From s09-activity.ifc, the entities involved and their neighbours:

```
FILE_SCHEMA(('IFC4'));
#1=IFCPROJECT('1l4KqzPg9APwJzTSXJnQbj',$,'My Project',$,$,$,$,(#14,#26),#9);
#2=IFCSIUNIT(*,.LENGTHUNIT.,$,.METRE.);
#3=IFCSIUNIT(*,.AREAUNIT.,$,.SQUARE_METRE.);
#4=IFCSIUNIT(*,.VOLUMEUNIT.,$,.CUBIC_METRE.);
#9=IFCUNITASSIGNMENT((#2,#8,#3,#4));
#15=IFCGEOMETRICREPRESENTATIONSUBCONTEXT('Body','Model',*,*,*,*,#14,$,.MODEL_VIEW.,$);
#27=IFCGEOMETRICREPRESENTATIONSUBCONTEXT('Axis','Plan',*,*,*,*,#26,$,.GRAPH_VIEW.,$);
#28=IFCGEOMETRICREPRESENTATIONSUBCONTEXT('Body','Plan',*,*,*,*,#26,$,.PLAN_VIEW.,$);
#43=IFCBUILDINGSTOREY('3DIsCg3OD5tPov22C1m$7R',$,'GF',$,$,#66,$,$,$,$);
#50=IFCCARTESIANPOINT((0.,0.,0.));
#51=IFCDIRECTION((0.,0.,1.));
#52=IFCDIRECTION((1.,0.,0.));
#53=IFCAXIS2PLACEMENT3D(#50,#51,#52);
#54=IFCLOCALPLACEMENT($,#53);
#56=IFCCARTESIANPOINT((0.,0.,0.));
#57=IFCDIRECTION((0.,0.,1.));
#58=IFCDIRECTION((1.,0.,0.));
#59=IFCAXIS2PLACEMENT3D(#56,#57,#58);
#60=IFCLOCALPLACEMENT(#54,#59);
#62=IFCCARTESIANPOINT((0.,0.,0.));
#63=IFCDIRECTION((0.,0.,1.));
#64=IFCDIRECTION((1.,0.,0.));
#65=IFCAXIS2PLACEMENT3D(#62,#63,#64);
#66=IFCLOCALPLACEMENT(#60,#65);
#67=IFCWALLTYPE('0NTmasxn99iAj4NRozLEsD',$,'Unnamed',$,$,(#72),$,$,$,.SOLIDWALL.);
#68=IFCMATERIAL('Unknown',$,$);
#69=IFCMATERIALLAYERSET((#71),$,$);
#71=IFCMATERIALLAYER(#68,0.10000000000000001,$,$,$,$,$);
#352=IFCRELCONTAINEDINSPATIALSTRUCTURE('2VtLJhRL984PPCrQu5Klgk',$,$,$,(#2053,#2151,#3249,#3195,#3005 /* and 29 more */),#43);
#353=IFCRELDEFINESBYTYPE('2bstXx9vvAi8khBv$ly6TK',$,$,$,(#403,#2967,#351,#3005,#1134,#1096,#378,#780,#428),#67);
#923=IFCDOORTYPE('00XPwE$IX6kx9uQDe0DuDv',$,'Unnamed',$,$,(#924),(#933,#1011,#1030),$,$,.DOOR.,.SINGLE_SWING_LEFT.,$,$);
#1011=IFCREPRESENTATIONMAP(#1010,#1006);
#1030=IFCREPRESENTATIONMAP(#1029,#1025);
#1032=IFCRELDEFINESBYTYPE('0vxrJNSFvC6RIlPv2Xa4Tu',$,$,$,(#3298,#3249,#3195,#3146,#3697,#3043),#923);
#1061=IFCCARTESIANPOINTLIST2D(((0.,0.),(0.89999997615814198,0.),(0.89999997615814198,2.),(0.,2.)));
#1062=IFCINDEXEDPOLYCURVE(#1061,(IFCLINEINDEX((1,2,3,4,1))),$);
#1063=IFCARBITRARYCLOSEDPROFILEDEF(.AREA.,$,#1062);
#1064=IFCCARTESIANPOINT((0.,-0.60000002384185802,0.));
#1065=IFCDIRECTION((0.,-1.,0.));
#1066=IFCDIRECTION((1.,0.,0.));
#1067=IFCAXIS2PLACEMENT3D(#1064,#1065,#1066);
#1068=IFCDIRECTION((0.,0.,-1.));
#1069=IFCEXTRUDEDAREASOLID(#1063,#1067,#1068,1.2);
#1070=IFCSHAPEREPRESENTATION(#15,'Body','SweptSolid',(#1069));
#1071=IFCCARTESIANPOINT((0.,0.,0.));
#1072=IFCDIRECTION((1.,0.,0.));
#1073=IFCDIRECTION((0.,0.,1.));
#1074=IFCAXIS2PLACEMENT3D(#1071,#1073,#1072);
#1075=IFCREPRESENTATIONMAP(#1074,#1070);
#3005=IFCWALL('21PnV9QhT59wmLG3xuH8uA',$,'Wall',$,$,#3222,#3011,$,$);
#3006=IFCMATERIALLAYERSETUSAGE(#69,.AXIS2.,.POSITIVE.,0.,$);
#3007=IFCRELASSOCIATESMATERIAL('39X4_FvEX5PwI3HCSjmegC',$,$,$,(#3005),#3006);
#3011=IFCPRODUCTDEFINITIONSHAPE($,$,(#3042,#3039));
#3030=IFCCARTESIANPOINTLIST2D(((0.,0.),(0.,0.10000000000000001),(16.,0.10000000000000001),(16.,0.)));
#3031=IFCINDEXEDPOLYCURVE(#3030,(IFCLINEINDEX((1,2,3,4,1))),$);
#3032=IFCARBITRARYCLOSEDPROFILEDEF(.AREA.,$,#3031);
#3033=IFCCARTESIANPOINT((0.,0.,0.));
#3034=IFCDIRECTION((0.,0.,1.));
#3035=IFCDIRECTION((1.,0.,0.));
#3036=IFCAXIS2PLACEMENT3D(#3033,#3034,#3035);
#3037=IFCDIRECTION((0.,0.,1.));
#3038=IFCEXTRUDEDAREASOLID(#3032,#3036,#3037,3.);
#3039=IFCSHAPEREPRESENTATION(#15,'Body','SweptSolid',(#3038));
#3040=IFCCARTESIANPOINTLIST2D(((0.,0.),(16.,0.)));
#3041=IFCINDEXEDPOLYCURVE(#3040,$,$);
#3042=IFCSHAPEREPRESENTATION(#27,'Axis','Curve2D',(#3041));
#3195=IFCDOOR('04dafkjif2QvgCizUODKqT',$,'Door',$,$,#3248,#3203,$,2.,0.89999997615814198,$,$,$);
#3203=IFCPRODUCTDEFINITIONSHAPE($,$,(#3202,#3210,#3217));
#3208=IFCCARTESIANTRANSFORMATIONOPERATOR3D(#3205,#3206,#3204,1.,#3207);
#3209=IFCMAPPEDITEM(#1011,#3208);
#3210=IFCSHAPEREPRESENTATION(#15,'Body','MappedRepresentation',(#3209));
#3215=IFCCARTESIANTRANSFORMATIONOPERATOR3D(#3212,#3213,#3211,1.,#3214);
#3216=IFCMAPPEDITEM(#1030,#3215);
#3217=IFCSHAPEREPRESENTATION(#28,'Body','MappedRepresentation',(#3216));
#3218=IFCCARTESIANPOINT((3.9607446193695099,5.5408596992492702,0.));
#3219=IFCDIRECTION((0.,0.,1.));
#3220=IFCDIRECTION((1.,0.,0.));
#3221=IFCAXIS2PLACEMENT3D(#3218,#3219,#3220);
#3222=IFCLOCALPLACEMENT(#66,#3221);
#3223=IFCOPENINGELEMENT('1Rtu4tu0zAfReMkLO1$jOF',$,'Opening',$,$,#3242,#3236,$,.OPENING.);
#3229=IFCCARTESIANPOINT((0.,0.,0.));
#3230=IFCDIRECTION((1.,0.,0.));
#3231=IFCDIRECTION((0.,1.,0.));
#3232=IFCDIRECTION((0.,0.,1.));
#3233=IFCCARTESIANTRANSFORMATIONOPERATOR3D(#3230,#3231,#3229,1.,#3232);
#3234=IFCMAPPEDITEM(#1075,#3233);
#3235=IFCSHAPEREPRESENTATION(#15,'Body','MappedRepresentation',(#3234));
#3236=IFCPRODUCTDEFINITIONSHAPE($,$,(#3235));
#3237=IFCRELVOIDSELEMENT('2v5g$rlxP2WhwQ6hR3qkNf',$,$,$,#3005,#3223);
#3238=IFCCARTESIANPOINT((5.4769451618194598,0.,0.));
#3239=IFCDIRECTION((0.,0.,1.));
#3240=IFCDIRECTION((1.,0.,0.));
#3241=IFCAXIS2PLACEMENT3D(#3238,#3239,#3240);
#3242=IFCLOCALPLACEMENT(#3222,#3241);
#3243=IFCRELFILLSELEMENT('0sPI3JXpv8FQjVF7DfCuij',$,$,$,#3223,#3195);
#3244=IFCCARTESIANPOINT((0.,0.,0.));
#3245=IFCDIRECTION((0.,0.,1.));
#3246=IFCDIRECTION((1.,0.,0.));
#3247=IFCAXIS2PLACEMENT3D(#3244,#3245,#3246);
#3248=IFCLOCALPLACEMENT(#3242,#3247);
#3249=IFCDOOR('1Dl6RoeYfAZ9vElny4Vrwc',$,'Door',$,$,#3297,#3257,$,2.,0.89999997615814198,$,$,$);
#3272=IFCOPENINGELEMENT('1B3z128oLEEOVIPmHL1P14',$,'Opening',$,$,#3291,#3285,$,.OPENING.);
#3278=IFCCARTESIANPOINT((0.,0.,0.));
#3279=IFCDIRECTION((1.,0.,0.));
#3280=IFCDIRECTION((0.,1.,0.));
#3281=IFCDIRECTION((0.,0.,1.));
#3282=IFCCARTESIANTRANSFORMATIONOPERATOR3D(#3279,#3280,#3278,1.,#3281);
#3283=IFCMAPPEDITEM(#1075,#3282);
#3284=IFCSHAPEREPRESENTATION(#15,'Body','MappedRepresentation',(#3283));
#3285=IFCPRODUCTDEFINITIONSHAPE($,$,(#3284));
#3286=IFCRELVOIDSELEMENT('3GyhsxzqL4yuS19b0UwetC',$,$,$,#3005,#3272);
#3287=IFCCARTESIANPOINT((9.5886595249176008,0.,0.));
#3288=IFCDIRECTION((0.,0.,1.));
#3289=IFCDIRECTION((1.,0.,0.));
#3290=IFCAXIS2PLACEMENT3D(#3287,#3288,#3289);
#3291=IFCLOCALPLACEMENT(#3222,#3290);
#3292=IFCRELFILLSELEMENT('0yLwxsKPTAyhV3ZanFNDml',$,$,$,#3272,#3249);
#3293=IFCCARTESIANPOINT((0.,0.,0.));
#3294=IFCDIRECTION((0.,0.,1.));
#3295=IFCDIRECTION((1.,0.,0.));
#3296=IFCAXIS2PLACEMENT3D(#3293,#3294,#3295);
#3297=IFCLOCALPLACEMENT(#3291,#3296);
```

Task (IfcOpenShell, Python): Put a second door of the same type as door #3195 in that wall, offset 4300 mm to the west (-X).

```python
import ifcopenshell
import ifcopenshell.api.feature
import ifcopenshell.api.geometry
import ifcopenshell.api.root
import ifcopenshell.geom
import ifcopenshell.util.element
import ifcopenshell.util.placement
import ifcopenshell.util.shape
import ifcopenshell.util.unit

model = ifcopenshell.open("s09-activity.ifc")
unit_scale = ifcopenshell.util.unit.calculate_unit_scale(model)
settings = ifcopenshell.geom.settings()


def volume(element):
    """Net volume in cubic metres, openings subtracted."""
    shape = ifcopenshell.geom.create_shape(settings, element)
    return ifcopenshell.util.shape.get_volume(shape.geometry)


door = model.by_guid("04dafkjif2QvgCizUODKqT")
opening = door.FillsVoids[0].RelatingOpeningElement
wall = opening.VoidsElements[0].RelatingBuildingElement
before = volume(wall)
shift = ifcopenshell.util.placement.get_local_placement(wall.ObjectPlacement)[:3, 0] * -4.3 / unit_scale

# copy_class copies the void relationship, type, container and properties, but no geometry.
new_opening = ifcopenshell.api.root.copy_class(model, product=opening)
new_opening.Representation = ifcopenshell.util.element.copy_deep(
    model, opening.Representation, exclude=["IfcGeometricRepresentationContext", "IfcRepresentationMap"]
)
new_door = ifcopenshell.api.root.copy_class(model, product=door)
new_door.Representation = ifcopenshell.util.element.copy_deep(
    model, door.Representation, exclude=["IfcGeometricRepresentationContext", "IfcRepresentationMap"]
)
ifcopenshell.api.feature.add_filling(model, opening=new_opening, element=new_door)

for old, new in ((opening, new_opening), (door, new_door)):
    matrix = ifcopenshell.util.placement.get_local_placement(old.ObjectPlacement)
    matrix[:3, 3] += shift
    ifcopenshell.api.geometry.edit_object_placement(model, product=new, matrix=matrix, is_si=False)

after = volume(wall)

print(f"wall volume {before:.3f} -> {after:.3f} m3")

model.write("s09-activity_v2.ifc")
```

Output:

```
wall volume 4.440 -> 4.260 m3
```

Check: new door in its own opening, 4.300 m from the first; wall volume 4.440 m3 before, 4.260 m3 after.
